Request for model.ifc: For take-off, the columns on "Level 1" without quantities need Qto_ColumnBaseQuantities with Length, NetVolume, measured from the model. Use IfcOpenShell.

First a look at what the model holds.

```python
import ifcopenshell
import ifcopenshell.util.element
import ifcopenshell.util.unit

model = ifcopenshell.open("model.ifc")
print(model.schema)
for unit_type in ("LENGTHUNIT", "AREAUNIT", "VOLUMEUNIT"):
    print(unit_type, ifcopenshell.util.unit.calculate_unit_scale(model, unit_type))
storey = next(s for s in model.by_type("IfcBuildingStorey") if s.Name == "Level 1")
columns = [e for e in ifcopenshell.util.element.get_decomposition(storey) if e.is_a("IfcColumn")]
for e in sorted(columns, key=lambda e: e.id()):
    print(e.id(), e.is_a(), e.Name, list(ifcopenshell.util.element.get_psets(e, qtos_only=True)), sep=" | ")
```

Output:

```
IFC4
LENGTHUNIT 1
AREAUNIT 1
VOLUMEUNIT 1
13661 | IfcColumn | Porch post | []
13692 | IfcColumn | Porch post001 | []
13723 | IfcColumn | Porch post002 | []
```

```python
import ifcopenshell
import ifcopenshell.api.pset
import ifcopenshell.geom
import ifcopenshell.util.element
import ifcopenshell.util.shape
import ifcopenshell.util.unit

model = ifcopenshell.open("model.ifc")
unit_scale = ifcopenshell.util.unit.calculate_unit_scale(model)
volume_scale = ifcopenshell.util.unit.calculate_unit_scale(model, "VOLUMEUNIT")
settings = ifcopenshell.geom.settings()

storey = next(s for s in model.by_type("IfcBuildingStorey") if s.Name == "Level 1")
columns = [e for e in ifcopenshell.util.element.get_decomposition(storey) if e.is_a("IfcColumn")]

for e in sorted(columns, key=lambda e: e.id()):
    if ifcopenshell.util.element.get_psets(e, qtos_only=True, should_inherit=False):
        continue
    # Geometry comes back in metres, in the element's own axes.
    shape = ifcopenshell.geom.create_shape(settings, e)
    values = {
        "Length": ifcopenshell.util.shape.get_z(shape.geometry) / unit_scale,
        "NetVolume": ifcopenshell.util.shape.get_volume(shape.geometry) / volume_scale,
    }
    qto = ifcopenshell.api.pset.add_qto(model, product=e, name="Qto_ColumnBaseQuantities")
    ifcopenshell.api.pset.edit_qto(model, qto=qto, properties=values)
    print(e.id(), {k: round(v, 3) for k, v in values.items()})

model.write("model_edited.ifc")
```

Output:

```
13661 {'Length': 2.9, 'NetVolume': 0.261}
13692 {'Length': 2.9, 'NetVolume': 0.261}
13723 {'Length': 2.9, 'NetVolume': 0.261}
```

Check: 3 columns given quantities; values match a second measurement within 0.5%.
